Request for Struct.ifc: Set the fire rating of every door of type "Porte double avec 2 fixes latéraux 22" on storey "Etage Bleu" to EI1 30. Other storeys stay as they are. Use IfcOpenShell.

First a look at what the model holds.

```python
import ifcopenshell
import ifcopenshell.util.element

model = ifcopenshell.open("Struct.ifc")
print(model.schema)
storey = next(s for s in model.by_type("IfcBuildingStorey") if s.Name == "Etage Bleu")
doors = [e for e in ifcopenshell.util.element.get_decomposition(storey) if e.is_a("IfcDoor")]
seen = {}
for e in doors:
    element_type = ifcopenshell.util.element.get_type(e)
    key = (element_type.Name if element_type != e and element_type else None, ifcopenshell.util.element.get_pset(e, "Pset_DoorCommon", "FireRating"))
    seen[key] = seen.get(key, 0) + 1
for (name, value), count in sorted(seen.items(), key=str):
    print(count, "x", name, "|", value)
```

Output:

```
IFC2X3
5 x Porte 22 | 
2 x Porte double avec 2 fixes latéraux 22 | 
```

```python
import ifcopenshell
import ifcopenshell.api.pset
import ifcopenshell.util.element

model = ifcopenshell.open("Struct.ifc")

storey = next(s for s in model.by_type("IfcBuildingStorey") if s.Name == "Etage Bleu")
doors = [e for e in ifcopenshell.util.element.get_decomposition(storey) if e.is_a("IfcDoor")]

count = 0
for e in doors:
    element_type = ifcopenshell.util.element.get_type(e)
    if element_type in (None, e) or element_type.Name != "Porte double avec 2 fixes latéraux 22":
        continue
    # add_pset returns the element's existing set when there is one.
    pset = ifcopenshell.api.pset.add_pset(model, product=e, name="Pset_DoorCommon")
    ifcopenshell.api.pset.edit_pset(model, pset=pset, properties={"FireRating": "EI1 30"})
    count += 1

print(count, "doors updated")

model.write("Struct_edited.ifc")
```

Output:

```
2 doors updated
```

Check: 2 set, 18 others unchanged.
